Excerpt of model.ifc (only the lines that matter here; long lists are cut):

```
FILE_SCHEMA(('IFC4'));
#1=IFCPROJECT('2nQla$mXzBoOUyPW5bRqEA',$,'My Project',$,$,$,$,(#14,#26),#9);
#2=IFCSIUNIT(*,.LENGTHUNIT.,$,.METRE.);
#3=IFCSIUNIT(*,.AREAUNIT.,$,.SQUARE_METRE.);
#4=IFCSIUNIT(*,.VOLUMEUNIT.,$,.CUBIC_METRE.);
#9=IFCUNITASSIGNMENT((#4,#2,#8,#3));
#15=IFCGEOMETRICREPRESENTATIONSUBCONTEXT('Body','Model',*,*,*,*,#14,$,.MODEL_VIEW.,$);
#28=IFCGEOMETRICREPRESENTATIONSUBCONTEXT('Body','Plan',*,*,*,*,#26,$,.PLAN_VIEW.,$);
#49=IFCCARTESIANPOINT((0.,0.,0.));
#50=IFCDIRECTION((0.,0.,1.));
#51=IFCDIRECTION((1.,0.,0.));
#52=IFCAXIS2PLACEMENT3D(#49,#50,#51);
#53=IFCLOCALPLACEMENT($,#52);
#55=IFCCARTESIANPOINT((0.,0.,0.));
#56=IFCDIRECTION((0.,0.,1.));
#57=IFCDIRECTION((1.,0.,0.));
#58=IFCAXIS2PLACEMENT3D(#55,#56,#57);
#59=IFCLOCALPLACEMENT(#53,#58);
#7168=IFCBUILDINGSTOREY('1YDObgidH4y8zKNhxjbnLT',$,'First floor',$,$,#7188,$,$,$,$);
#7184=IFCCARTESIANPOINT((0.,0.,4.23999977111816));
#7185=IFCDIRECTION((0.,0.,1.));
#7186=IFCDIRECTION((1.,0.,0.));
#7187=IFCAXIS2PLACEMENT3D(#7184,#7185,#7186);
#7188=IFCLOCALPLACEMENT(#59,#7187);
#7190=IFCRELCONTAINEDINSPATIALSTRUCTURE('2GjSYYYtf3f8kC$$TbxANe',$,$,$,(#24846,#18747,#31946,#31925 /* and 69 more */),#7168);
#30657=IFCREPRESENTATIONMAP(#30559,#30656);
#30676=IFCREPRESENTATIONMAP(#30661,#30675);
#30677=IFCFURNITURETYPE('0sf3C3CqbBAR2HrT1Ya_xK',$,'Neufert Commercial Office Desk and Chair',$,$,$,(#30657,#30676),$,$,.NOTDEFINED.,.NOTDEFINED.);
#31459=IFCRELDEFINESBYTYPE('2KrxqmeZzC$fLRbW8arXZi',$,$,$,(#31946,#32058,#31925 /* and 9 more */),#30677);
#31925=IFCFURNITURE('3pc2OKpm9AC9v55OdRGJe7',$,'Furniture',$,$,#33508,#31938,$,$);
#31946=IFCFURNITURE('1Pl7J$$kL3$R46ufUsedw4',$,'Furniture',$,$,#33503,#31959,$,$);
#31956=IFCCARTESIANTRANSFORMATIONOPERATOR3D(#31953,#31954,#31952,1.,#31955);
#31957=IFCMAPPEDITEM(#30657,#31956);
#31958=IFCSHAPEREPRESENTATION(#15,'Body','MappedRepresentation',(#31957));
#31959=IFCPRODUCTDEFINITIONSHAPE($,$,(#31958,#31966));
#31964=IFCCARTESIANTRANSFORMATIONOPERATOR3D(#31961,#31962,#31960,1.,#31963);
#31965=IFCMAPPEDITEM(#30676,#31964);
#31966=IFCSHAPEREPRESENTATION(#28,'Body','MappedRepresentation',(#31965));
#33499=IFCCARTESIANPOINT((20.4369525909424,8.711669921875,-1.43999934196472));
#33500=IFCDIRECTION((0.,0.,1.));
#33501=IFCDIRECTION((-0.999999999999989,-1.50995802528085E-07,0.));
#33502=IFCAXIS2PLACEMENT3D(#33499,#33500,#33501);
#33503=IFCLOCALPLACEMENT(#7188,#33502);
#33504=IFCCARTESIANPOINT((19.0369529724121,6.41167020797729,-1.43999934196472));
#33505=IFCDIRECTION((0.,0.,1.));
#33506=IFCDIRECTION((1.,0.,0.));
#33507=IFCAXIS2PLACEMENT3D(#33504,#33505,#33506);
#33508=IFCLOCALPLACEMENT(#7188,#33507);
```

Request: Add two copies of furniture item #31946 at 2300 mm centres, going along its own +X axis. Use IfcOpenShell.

```python
import ifcopenshell
import ifcopenshell.api.geometry
import ifcopenshell.api.root
import ifcopenshell.util.element
import ifcopenshell.util.placement
import ifcopenshell.util.unit

model = ifcopenshell.open("model.ifc")
unit_scale = ifcopenshell.util.unit.calculate_unit_scale(model)

source = model.by_id(31946)
base = ifcopenshell.util.placement.get_local_placement(source.ObjectPlacement)
step = base[:3, 0] * 2.3 / unit_scale

for i in range(1, 3):
    copy = ifcopenshell.api.root.copy_class(model, product=source)
    copy.Representation = ifcopenshell.util.element.copy_deep(
        model, source.Representation, exclude=["IfcGeometricRepresentationContext", "IfcRepresentationMap"]
    )
    matrix = base.copy()
    matrix[:3, 3] += i * step
    print("added at", matrix[:3, 3].round(3) + 0.0)
    ifcopenshell.api.geometry.edit_object_placement(model, product=copy, matrix=matrix, is_si=False)

model.write("model-out.ifc")
```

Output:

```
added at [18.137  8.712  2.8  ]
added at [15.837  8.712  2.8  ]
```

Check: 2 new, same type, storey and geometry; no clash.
